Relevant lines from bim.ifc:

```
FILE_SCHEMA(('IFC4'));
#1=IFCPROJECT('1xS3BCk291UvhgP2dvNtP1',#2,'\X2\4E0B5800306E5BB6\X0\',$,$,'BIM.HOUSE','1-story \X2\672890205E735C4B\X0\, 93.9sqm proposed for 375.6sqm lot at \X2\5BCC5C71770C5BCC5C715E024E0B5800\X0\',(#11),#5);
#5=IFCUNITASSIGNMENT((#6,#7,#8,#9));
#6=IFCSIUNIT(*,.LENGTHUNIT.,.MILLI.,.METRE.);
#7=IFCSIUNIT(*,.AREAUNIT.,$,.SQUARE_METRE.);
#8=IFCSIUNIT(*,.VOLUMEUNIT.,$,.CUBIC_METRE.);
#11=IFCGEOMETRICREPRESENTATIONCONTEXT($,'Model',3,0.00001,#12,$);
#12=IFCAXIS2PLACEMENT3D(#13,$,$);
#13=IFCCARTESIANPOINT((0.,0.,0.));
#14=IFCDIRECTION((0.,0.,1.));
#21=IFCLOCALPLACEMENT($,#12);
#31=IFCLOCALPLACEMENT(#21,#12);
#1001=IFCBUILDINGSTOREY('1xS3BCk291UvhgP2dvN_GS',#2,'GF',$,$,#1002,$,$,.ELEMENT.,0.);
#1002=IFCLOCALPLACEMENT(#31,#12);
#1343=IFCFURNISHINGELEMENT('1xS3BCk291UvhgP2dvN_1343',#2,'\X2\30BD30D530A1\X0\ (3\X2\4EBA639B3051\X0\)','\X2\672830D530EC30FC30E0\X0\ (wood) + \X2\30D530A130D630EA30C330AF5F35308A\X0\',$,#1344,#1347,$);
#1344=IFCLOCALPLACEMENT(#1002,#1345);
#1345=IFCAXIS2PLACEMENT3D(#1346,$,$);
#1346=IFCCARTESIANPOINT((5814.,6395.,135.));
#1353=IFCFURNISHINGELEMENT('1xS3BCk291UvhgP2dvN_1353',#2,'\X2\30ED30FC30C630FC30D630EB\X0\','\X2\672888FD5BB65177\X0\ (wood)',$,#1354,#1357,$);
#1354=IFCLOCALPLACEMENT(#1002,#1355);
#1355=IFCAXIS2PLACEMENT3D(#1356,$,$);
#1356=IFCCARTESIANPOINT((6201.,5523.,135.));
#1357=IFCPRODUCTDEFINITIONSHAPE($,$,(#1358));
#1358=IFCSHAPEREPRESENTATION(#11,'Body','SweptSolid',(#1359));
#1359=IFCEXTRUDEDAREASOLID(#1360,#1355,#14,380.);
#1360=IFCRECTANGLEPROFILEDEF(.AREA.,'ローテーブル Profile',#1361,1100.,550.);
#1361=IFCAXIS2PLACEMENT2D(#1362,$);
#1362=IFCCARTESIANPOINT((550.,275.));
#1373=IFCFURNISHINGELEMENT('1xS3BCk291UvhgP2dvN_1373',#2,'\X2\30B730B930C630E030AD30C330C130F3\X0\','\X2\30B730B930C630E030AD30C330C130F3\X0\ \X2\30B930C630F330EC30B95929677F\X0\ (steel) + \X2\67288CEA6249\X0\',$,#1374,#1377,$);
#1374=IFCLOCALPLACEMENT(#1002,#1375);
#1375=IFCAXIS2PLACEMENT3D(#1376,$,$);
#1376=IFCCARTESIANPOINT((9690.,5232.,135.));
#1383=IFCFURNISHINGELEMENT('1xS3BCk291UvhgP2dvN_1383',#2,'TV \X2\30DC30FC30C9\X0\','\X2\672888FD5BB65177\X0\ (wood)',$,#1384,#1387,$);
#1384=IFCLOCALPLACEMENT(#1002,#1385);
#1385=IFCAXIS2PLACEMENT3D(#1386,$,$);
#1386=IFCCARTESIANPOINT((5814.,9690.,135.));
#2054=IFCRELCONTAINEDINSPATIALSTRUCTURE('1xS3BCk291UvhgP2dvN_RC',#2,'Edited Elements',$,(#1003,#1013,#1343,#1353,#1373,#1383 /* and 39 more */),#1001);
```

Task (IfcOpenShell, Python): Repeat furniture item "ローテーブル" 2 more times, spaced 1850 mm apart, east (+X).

```python
import numpy as np
import ifcopenshell
import ifcopenshell.api.geometry
import ifcopenshell.api.root
import ifcopenshell.util.element
import ifcopenshell.util.placement

model = ifcopenshell.open("bim.ifc")


def reuse_history(source, copy):
    """copy_class also copies each property set's owner history, people and application; keep the originals."""
    for rel in copy.IsDefinedBy:
        if rel.is_a("IfcRelDefinesByProperties") and (history := rel.RelatingPropertyDefinition.OwnerHistory):
            rel.RelatingPropertyDefinition.OwnerHistory = source.OwnerHistory
            ifcopenshell.util.element.remove_deep2(model, history)


source = model.by_guid("1xS3BCk291UvhgP2dvN_1353")
base = ifcopenshell.util.placement.get_local_placement(source.ObjectPlacement)
step = np.array([1.0, 0.0, 0.0]) * 1850.0

for i in range(1, 3):
    copy = ifcopenshell.api.root.copy_class(model, product=source)
    copy.Representation = ifcopenshell.util.element.copy_deep(
        model, source.Representation, exclude=["IfcGeometricRepresentationContext", "IfcRepresentationMap"]
    )
    reuse_history(source, copy)
    matrix = base.copy()
    matrix[:3, 3] += i * step
    print("added at", matrix[:3, 3].round(3) + 0.0)
    ifcopenshell.api.geometry.edit_object_placement(model, product=copy, matrix=matrix, is_si=False)

model.write("bim_v2.ifc")
```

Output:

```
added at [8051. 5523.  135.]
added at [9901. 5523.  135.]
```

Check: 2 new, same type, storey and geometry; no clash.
